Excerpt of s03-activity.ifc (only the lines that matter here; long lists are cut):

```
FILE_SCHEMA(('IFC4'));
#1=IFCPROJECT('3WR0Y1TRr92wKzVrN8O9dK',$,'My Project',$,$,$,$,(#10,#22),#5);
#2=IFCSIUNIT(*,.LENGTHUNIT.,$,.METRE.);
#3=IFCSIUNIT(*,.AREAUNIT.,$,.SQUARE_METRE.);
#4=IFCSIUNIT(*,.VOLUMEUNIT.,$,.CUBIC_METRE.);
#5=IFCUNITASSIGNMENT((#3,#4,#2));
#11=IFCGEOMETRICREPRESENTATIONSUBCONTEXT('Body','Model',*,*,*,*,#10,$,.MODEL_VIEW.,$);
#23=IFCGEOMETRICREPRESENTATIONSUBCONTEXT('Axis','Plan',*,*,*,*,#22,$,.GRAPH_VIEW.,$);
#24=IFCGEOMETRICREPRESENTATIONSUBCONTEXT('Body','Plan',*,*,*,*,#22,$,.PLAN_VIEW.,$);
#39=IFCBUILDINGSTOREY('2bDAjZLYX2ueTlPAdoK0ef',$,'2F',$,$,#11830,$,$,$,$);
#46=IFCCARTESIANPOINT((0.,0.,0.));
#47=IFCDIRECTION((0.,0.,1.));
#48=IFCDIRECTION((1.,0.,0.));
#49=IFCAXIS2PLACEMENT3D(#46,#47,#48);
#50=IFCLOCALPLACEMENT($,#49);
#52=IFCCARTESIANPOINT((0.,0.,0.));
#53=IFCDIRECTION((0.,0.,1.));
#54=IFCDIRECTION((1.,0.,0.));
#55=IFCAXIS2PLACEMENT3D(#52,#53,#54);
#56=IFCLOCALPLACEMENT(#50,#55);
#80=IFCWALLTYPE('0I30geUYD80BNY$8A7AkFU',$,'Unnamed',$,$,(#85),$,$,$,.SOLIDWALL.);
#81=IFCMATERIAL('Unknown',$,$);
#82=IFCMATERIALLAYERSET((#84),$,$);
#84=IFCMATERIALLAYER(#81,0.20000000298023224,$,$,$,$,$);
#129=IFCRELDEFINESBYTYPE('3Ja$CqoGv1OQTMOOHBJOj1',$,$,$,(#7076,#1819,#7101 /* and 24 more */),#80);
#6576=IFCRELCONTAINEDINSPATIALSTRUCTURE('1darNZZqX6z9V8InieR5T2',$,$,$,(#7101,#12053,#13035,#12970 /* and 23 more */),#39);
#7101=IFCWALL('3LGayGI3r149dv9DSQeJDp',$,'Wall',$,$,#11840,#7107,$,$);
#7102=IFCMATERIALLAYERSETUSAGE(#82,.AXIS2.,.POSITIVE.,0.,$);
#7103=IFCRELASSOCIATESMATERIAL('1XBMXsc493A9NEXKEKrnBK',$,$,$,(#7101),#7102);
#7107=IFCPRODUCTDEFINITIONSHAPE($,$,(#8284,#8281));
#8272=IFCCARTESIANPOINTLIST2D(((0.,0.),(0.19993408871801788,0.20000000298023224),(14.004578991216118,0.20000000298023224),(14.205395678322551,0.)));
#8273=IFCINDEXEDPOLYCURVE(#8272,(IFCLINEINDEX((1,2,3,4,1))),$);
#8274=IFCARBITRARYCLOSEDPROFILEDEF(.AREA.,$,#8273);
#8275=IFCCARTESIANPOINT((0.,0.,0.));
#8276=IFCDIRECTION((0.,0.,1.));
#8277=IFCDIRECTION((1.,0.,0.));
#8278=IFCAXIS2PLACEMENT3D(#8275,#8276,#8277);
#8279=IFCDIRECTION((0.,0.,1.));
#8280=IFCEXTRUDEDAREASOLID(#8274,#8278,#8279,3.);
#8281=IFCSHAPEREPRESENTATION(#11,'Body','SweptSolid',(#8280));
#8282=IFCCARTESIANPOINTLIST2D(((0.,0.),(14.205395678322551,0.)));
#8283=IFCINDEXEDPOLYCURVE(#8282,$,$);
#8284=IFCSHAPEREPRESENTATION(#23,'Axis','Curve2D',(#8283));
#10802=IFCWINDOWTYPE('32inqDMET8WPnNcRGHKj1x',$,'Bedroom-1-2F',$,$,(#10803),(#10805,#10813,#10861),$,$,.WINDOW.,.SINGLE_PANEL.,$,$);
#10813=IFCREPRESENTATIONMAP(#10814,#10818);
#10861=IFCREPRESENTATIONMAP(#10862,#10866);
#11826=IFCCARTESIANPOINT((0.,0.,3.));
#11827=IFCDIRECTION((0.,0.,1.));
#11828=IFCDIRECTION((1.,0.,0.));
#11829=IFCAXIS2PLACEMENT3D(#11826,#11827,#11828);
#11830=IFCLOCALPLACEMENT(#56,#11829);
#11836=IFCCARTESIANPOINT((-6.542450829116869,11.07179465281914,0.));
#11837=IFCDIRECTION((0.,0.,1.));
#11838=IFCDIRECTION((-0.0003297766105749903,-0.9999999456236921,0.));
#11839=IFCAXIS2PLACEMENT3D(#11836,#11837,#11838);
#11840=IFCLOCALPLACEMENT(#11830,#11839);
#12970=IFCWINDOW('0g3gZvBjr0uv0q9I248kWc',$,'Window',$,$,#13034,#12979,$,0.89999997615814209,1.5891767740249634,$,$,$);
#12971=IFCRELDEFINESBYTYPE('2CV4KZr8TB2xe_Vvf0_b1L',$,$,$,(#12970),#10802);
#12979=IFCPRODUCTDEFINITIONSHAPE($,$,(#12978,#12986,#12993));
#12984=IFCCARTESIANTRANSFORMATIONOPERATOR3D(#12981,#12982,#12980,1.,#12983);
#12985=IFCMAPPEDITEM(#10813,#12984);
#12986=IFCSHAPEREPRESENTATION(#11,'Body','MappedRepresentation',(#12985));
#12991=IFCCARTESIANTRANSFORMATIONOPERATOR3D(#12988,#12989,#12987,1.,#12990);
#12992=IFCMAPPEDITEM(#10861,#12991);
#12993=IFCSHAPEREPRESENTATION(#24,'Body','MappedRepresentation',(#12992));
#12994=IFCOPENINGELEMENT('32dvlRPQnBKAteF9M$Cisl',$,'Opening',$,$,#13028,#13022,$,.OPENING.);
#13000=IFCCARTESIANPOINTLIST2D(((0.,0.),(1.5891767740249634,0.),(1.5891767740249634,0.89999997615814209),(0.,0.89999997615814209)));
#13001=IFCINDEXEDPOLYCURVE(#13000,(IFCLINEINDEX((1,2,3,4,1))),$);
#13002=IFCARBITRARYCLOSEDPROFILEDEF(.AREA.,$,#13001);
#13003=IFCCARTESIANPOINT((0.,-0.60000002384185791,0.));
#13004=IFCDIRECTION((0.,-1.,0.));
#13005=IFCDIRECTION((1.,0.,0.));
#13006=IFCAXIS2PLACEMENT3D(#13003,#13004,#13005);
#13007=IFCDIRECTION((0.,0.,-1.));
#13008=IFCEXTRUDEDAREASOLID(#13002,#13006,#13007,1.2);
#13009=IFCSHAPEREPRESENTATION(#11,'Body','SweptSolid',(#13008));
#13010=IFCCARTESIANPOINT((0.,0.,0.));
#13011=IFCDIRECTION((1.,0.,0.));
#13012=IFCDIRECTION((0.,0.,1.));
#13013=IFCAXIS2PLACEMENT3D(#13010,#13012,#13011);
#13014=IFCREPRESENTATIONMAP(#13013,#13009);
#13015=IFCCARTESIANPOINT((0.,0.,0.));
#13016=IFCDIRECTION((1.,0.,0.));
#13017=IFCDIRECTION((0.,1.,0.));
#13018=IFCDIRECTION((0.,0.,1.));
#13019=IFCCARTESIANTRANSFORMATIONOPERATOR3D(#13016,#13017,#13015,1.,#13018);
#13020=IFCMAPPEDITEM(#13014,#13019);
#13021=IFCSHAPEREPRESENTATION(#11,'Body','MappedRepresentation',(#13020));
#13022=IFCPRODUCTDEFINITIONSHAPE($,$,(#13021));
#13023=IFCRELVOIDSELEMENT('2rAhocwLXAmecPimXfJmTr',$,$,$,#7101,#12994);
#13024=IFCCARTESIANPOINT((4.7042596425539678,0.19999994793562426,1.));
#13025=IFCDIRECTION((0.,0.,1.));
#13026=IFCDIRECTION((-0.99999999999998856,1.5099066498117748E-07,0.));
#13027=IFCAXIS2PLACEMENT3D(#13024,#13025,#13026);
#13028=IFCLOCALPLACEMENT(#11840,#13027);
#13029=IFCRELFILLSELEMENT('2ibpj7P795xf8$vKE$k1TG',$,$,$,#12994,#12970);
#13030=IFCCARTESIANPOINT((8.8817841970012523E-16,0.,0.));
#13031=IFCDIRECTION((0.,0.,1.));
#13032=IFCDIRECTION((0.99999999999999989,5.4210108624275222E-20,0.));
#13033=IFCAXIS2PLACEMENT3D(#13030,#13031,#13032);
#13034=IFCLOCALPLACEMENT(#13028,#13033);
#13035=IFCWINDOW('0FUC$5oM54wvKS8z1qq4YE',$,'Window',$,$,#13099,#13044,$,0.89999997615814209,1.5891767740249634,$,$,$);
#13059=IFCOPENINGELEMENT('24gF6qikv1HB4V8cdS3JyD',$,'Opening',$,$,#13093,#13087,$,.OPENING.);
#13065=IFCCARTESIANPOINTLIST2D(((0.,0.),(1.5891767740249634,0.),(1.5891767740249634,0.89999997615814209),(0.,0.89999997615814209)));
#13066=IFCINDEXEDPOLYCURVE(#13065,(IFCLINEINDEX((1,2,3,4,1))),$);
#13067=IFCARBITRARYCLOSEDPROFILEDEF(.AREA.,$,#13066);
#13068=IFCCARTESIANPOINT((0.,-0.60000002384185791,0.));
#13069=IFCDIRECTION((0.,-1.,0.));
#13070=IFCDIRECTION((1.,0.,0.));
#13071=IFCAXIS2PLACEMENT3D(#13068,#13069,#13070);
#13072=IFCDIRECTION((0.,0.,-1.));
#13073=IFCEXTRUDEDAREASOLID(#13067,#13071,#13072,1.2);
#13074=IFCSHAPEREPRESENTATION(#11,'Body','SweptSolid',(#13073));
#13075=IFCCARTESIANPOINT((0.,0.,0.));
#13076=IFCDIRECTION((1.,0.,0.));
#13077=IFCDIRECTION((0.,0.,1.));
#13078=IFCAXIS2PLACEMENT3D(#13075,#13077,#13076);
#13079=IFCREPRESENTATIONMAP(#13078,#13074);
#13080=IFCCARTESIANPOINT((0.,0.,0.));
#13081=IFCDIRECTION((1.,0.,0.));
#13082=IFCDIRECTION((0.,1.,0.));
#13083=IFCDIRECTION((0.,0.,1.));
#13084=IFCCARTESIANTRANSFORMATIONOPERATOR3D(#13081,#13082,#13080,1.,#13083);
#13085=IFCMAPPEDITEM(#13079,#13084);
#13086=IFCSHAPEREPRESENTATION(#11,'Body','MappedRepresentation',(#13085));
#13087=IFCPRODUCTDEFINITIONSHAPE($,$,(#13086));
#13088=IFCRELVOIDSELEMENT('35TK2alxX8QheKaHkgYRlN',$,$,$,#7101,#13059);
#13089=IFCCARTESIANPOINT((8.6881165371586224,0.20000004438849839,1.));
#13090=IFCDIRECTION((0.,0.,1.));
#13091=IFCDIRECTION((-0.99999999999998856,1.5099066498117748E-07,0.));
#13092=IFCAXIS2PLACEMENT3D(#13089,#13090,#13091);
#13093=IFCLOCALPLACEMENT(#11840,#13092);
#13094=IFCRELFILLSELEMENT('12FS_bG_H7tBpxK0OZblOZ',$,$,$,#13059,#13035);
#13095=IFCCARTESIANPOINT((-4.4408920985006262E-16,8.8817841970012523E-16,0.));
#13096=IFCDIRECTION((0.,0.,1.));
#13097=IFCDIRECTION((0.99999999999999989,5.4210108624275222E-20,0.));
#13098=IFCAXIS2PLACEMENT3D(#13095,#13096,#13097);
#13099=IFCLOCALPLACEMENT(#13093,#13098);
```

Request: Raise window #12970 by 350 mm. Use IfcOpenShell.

```python
import numpy as np
import ifcopenshell
import ifcopenshell.api.geometry
import ifcopenshell.util.placement
import ifcopenshell.util.unit

model = ifcopenshell.open("s03-activity.ifc")
unit_scale = ifcopenshell.util.unit.calculate_unit_scale(model)

window = model.by_guid("0g3gZvBjr0uv0q9I248kWc")
opening = window.FillsVoids[0].RelatingOpeningElement
dz = 0.35

shift = np.array([0.0, 0.0, dz])
# The window is placed relative to its opening, so it follows when the opening moves.
matrix = ifcopenshell.util.placement.get_local_placement(opening.ObjectPlacement)
matrix[:3, 3] += shift
ifcopenshell.api.geometry.edit_object_placement(
    model, product=opening, matrix=matrix, is_si=False, should_transform_children=True
)

print(f"moved by {dz * unit_scale:+.3f} m")

model.write("s03-activity_updated.ifc")
```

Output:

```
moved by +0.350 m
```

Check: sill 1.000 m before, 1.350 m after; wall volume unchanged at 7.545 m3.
